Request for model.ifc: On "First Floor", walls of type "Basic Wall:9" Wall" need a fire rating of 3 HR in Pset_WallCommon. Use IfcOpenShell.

First a look at what the model holds.

```python
import ifcopenshell
import ifcopenshell.util.element

model = ifcopenshell.open("model.ifc")
print(model.schema)
storey = next(s for s in model.by_type("IfcBuildingStorey") if s.Name == "First Floor")
walls = [e for e in ifcopenshell.util.element.get_decomposition(storey) if e.is_a("IfcWall")]
seen = {}
for e in walls:
    element_type = ifcopenshell.util.element.get_type(e)
    key = (element_type.Name if element_type != e and element_type else None, ifcopenshell.util.element.get_pset(e, "Pset_WallCommon", "FireRating"))
    seen[key] = seen.get(key, 0) + 1
for (name, value), count in sorted(seen.items(), key=str):
    print(count, "x", name, "|", value)
```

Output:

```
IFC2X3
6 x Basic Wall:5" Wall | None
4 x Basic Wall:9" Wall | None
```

```python
import ifcopenshell
import ifcopenshell.api.pset
import ifcopenshell.util.element

model = ifcopenshell.open("model.ifc")

storey = next(s for s in model.by_type("IfcBuildingStorey") if s.Name == "First Floor")
walls = [e for e in ifcopenshell.util.element.get_decomposition(storey) if e.is_a("IfcWall")]

count = 0
for e in walls:
    element_type = ifcopenshell.util.element.get_type(e)
    if element_type in (None, e) or element_type.Name != 'Basic Wall:9" Wall':
        continue
    # add_pset returns the element's existing set when there is one.
    pset = ifcopenshell.api.pset.add_pset(model, product=e, name="Pset_WallCommon")
    ifcopenshell.api.pset.edit_pset(model, pset=pset, properties={"FireRating": "3 HR"})
    count += 1

print(count, "walls updated")

model.write("model-out.ifc")
```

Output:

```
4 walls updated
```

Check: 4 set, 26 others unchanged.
